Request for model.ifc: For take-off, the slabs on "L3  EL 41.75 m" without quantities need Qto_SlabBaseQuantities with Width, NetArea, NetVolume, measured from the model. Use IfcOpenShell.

First a look at what the model holds.

```python
import ifcopenshell
import ifcopenshell.util.element
import ifcopenshell.util.unit

model = ifcopenshell.open("model.ifc")
print(model.schema)
for unit_type in ("LENGTHUNIT", "AREAUNIT", "VOLUMEUNIT"):
    print(unit_type, ifcopenshell.util.unit.calculate_unit_scale(model, unit_type))
storey = next(s for s in model.by_type("IfcBuildingStorey") if s.Name == "L3  EL 41.75 m")
slabs = [e for e in ifcopenshell.util.element.get_decomposition(storey) if e.is_a("IfcSlab")]
for e in sorted(slabs, key=lambda e: e.id()):
    print(e.id(), e.is_a(), e.Name, list(ifcopenshell.util.element.get_psets(e, qtos_only=True)), sep=" | ")
```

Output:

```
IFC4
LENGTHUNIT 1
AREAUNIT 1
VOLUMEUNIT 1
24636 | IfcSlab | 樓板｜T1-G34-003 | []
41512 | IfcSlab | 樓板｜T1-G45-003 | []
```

```python
import ifcopenshell
import ifcopenshell.api.pset
import ifcopenshell.geom
import ifcopenshell.util.element
import ifcopenshell.util.shape
import ifcopenshell.util.unit

model = ifcopenshell.open("model.ifc")
unit_scale = ifcopenshell.util.unit.calculate_unit_scale(model)
area_scale = ifcopenshell.util.unit.calculate_unit_scale(model, "AREAUNIT")
volume_scale = ifcopenshell.util.unit.calculate_unit_scale(model, "VOLUMEUNIT")
settings = ifcopenshell.geom.settings()

storey = next(s for s in model.by_type("IfcBuildingStorey") if s.Name == "L3  EL 41.75 m")
slabs = [e for e in ifcopenshell.util.element.get_decomposition(storey) if e.is_a("IfcSlab")]

for e in sorted(slabs, key=lambda e: e.id()):
    if ifcopenshell.util.element.get_psets(e, qtos_only=True, should_inherit=False):
        continue
    # Geometry comes back in metres, in the element's own axes.
    shape = ifcopenshell.geom.create_shape(settings, e)
    values = {
        "Width": ifcopenshell.util.shape.get_z(shape.geometry) / unit_scale,
        "NetArea": ifcopenshell.util.shape.get_footprint_area(shape.geometry) / area_scale,
        "NetVolume": ifcopenshell.util.shape.get_volume(shape.geometry) / volume_scale,
    }
    qto = ifcopenshell.api.pset.add_qto(model, product=e, name="Qto_SlabBaseQuantities")
    ifcopenshell.api.pset.edit_qto(model, qto=qto, properties=values)
    print(e.id(), {k: round(v, 3) for k, v in values.items()})

model.write("model-out.ifc")
```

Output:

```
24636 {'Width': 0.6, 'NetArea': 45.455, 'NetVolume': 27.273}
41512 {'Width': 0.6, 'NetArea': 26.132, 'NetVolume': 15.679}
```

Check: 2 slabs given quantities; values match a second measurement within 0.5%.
